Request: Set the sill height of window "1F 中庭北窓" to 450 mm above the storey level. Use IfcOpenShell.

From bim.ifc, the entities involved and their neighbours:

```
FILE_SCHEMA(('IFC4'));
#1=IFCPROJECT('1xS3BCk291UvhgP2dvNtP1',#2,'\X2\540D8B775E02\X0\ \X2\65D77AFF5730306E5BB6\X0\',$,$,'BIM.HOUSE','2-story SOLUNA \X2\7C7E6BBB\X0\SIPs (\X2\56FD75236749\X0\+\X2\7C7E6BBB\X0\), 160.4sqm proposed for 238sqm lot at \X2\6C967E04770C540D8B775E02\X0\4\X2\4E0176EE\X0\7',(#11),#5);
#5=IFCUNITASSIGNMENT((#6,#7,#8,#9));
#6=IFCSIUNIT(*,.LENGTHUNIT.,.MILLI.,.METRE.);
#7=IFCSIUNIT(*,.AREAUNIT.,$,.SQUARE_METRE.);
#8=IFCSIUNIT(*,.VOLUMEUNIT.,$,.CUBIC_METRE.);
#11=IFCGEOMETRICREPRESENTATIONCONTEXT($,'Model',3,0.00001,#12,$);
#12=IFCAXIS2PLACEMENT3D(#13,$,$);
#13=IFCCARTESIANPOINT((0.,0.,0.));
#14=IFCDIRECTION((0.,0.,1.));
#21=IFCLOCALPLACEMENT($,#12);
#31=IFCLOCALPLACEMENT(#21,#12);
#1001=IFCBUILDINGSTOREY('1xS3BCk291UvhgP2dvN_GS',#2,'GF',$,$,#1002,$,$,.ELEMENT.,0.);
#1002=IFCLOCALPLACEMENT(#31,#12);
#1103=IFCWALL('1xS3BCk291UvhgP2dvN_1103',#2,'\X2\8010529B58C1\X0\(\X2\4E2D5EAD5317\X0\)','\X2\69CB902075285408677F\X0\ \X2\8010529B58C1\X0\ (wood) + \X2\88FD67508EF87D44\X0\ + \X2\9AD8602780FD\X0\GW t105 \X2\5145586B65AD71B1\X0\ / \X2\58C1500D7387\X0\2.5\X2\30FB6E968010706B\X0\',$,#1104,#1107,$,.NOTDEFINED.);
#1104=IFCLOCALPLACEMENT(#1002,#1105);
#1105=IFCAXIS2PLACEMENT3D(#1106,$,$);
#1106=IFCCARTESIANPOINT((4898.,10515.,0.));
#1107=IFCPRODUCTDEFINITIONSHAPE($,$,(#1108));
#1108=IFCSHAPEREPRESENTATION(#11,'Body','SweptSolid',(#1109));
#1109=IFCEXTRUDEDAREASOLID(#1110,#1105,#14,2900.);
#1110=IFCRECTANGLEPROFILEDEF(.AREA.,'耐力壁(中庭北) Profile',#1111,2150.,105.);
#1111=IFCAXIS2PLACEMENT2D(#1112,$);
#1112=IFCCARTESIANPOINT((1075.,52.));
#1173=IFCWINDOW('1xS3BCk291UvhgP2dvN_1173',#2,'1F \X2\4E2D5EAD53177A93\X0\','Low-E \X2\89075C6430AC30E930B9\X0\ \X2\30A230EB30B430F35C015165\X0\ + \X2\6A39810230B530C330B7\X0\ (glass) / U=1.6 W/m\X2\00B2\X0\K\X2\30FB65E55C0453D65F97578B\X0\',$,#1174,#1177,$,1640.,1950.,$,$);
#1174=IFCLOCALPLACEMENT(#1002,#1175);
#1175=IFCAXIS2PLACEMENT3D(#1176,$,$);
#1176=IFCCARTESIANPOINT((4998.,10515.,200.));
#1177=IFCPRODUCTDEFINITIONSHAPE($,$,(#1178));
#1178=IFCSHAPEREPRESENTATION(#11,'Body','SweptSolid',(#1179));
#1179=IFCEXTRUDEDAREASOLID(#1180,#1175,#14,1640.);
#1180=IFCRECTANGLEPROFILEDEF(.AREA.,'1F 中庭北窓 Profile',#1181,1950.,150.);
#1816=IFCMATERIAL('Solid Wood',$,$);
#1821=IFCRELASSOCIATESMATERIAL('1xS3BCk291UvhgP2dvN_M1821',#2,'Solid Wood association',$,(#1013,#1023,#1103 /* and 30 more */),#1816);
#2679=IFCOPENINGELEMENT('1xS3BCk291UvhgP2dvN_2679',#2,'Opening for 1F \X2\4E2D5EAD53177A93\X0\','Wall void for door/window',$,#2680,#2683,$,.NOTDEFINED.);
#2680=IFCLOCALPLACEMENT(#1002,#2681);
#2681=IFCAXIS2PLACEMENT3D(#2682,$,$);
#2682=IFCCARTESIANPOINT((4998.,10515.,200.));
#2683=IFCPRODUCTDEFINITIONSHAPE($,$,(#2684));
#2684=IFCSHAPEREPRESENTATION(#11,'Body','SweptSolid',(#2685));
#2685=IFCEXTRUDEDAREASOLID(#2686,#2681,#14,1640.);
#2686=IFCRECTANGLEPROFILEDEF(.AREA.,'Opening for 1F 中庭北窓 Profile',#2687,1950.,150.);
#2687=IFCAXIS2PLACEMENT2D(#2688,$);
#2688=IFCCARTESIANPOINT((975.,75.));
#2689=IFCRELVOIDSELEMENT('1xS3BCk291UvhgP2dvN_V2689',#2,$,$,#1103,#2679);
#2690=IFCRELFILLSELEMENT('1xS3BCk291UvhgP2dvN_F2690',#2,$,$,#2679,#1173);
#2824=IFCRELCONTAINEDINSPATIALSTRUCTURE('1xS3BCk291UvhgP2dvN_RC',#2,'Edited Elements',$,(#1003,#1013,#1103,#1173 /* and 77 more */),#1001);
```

```python
import numpy as np
import ifcopenshell
import ifcopenshell.api.geometry
import ifcopenshell.geom
import ifcopenshell.util.element
import ifcopenshell.util.placement
import ifcopenshell.util.shape
import ifcopenshell.util.unit

model = ifcopenshell.open("bim.ifc")
unit_scale = ifcopenshell.util.unit.calculate_unit_scale(model)

window = model.by_guid("1xS3BCk291UvhgP2dvN_1173")
opening = window.FillsVoids[0].RelatingOpeningElement
storey = ifcopenshell.util.element.get_container(window, ifc_class="IfcBuildingStorey")
level = ifcopenshell.util.placement.get_local_placement(storey.ObjectPlacement)[2, 3]

# The opening's origin need not be at the sill, so measure its lowest point.
shape = ifcopenshell.geom.create_shape(ifcopenshell.geom.settings(), opening)
bottom = ifcopenshell.util.shape.get_shape_bottom_elevation(shape, shape.geometry) / unit_scale
dz = level + 450.0 - bottom

shift = np.array([0.0, 0.0, dz])
# The window is not placed relative to its opening, so move both.
for product in (opening, window):
    matrix = ifcopenshell.util.placement.get_local_placement(product.ObjectPlacement)
    matrix[:3, 3] += shift
    ifcopenshell.api.geometry.edit_object_placement(model, product=product, matrix=matrix, is_si=False)

print(f"moved by {dz * unit_scale:+.3f} m")

model.write("bim_edited.ifc")
```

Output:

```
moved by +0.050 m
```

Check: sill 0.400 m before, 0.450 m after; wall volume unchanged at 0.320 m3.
